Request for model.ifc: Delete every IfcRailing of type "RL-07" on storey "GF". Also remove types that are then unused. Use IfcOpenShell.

First a look at what the model holds.

```python
import ifcopenshell
import ifcopenshell.util.element

model = ifcopenshell.open("model.ifc")
print(model.schema)
storey = next(s for s in model.by_type("IfcBuildingStorey") if s.Name == "GF")
railings = [e for e in ifcopenshell.util.element.get_decomposition(storey) if e.is_a("IfcRailing")]
seen = {}
for e in railings:
    element_type = ifcopenshell.util.element.get_type(e)
    name = element_type.Name if element_type not in (None, e) else None
    seen[name] = seen.get(name, 0) + 1
for name, count in sorted(seen.items(), key=str):
    print(count, "x", name)
```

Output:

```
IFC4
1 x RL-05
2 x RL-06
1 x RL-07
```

```python
import ifcopenshell
import ifcopenshell.api.root
import ifcopenshell.util.element

model = ifcopenshell.open("model.ifc")

storey = next(s for s in model.by_type("IfcBuildingStorey") if s.Name == "GF")
railings = [e for e in ifcopenshell.util.element.get_decomposition(storey) if e.is_a("IfcRailing")]
targets = [e for e in railings if (t := ifcopenshell.util.element.get_type(e)) not in (None, e) and t.Name == "RL-07"]
types = {ifcopenshell.util.element.get_type(e) for e in targets} - {None, *targets}

for e in targets:
    ifcopenshell.api.root.remove_product(model, product=e)
print(len(targets), "removed")

unused = [t for t in types if not ifcopenshell.util.element.get_types(t)]
for t in unused:
    ifcopenshell.api.root.remove_product(model, product=t)
print(len(unused), "unused types removed")

model.write("model_v2.ifc")
```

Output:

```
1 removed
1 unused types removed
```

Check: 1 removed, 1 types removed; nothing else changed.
